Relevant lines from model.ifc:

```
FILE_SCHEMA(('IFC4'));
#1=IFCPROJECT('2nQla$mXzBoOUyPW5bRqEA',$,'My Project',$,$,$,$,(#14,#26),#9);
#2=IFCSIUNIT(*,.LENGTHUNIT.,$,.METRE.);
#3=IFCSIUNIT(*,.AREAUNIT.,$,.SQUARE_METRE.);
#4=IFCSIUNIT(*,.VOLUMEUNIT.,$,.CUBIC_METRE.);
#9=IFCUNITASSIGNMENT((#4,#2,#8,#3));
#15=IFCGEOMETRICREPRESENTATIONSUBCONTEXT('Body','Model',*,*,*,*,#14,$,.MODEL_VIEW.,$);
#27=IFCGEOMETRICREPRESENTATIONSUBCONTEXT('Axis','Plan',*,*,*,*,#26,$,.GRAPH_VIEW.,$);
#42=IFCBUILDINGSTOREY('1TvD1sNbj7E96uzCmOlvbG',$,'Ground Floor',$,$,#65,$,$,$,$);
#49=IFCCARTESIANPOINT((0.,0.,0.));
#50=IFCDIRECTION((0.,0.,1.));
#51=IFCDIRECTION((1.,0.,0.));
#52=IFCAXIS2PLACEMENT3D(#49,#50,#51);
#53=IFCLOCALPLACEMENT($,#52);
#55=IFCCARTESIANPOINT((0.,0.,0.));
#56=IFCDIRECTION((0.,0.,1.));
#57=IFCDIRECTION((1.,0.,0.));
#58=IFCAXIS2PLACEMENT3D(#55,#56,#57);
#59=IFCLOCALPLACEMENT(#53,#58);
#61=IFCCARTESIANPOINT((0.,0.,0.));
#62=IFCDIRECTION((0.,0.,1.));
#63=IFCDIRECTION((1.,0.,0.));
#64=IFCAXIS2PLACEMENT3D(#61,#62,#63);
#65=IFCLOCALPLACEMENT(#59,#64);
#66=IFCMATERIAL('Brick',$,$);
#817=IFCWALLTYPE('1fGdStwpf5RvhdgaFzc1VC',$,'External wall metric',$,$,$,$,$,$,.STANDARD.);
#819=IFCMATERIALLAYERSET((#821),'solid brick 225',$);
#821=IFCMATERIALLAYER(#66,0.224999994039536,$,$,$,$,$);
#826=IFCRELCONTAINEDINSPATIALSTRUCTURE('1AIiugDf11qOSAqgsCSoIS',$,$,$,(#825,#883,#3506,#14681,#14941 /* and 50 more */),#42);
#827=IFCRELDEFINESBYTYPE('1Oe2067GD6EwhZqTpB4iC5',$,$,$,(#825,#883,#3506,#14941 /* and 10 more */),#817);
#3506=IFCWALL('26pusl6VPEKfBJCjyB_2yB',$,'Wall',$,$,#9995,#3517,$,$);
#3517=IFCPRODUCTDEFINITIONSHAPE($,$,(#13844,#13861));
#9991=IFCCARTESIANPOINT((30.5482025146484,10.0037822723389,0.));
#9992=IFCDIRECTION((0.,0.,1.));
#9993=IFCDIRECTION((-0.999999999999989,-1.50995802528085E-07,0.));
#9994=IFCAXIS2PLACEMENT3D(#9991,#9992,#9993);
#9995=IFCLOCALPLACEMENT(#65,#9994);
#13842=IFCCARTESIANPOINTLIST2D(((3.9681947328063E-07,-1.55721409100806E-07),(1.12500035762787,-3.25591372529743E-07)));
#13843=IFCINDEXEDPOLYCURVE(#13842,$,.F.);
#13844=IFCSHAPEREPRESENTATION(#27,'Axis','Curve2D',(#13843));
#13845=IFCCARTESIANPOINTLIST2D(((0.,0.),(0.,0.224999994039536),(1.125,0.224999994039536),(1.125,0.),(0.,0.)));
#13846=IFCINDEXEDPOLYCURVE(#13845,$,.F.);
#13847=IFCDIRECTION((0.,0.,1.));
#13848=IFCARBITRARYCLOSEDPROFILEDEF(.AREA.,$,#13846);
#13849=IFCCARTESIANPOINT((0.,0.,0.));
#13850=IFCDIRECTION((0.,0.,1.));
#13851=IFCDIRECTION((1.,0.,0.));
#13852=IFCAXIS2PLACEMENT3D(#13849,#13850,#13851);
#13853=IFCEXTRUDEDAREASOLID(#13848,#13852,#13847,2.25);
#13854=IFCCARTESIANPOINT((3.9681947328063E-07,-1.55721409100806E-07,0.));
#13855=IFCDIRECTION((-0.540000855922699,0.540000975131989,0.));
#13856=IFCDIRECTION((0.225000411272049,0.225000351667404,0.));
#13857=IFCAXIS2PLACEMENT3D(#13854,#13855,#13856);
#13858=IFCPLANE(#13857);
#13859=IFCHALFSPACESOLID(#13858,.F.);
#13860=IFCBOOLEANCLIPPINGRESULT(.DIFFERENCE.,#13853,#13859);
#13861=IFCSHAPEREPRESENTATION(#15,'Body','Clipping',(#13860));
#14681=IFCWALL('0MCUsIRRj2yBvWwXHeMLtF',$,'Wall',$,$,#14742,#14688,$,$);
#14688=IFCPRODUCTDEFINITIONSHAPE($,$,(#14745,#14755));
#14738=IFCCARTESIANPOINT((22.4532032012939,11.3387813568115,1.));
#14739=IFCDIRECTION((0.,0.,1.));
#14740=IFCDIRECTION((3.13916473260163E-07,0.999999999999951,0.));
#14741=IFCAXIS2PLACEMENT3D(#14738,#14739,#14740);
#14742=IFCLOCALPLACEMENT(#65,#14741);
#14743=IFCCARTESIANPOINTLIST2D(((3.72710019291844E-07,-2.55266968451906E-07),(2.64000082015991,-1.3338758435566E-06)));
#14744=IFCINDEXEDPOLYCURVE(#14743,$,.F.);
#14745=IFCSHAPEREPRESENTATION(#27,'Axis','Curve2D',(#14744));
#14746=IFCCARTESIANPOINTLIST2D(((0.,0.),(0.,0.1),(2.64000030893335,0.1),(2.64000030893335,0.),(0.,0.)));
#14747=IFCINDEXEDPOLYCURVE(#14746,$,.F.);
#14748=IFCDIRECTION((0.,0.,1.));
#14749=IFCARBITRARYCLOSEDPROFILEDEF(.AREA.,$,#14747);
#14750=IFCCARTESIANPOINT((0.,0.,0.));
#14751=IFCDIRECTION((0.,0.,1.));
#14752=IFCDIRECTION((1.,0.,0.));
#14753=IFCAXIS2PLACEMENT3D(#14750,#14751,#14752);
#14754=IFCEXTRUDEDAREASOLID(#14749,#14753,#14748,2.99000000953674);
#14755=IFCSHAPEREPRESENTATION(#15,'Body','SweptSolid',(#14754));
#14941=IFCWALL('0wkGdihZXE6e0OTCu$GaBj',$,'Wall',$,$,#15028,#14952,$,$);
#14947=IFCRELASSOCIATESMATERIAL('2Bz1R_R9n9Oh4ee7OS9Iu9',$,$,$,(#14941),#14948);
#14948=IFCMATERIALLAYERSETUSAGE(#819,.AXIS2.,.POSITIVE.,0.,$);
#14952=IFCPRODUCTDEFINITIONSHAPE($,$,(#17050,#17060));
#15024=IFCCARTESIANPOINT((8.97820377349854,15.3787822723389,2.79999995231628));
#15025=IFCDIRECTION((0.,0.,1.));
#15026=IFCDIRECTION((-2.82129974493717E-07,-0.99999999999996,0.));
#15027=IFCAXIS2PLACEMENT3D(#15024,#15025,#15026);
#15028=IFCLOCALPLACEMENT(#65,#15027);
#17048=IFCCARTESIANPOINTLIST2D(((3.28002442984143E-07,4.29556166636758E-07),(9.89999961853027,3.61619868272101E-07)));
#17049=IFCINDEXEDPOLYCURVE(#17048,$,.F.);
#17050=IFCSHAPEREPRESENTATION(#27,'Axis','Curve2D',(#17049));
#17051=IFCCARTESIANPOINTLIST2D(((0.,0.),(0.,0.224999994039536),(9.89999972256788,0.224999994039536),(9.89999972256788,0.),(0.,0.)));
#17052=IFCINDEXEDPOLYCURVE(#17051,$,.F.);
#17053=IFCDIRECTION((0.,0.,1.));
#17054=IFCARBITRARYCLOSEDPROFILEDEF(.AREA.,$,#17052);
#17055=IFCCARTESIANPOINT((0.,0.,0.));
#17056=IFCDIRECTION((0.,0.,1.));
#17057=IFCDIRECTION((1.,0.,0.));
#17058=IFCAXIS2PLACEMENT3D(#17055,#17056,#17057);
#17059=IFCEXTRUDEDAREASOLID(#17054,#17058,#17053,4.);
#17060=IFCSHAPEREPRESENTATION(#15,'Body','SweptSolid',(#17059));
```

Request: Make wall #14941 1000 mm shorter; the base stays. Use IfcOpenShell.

```python
import ifcopenshell
import ifcopenshell.geom
import ifcopenshell.util.representation
import ifcopenshell.util.shape

model = ifcopenshell.open("model.ifc")
settings = ifcopenshell.geom.settings()


def volume(element):
    """Net volume in cubic metres, openings subtracted."""
    shape = ifcopenshell.geom.create_shape(settings, element)
    return ifcopenshell.util.shape.get_volume(shape.geometry)


wall = model.by_id(14941)
before = volume(wall)

body = ifcopenshell.util.representation.get_representation(wall, "Model", "Body")
solid = body.Items[0]
old_height = solid.Depth
solid.Depth -= 1.0
after = volume(wall)

print(f"height {old_height:g} -> {solid.Depth:g}, volume {before:.3f} -> {after:.3f} m3")

model.write("model_rev.ifc")
```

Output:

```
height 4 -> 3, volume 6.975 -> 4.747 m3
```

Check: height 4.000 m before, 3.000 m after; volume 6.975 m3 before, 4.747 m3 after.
